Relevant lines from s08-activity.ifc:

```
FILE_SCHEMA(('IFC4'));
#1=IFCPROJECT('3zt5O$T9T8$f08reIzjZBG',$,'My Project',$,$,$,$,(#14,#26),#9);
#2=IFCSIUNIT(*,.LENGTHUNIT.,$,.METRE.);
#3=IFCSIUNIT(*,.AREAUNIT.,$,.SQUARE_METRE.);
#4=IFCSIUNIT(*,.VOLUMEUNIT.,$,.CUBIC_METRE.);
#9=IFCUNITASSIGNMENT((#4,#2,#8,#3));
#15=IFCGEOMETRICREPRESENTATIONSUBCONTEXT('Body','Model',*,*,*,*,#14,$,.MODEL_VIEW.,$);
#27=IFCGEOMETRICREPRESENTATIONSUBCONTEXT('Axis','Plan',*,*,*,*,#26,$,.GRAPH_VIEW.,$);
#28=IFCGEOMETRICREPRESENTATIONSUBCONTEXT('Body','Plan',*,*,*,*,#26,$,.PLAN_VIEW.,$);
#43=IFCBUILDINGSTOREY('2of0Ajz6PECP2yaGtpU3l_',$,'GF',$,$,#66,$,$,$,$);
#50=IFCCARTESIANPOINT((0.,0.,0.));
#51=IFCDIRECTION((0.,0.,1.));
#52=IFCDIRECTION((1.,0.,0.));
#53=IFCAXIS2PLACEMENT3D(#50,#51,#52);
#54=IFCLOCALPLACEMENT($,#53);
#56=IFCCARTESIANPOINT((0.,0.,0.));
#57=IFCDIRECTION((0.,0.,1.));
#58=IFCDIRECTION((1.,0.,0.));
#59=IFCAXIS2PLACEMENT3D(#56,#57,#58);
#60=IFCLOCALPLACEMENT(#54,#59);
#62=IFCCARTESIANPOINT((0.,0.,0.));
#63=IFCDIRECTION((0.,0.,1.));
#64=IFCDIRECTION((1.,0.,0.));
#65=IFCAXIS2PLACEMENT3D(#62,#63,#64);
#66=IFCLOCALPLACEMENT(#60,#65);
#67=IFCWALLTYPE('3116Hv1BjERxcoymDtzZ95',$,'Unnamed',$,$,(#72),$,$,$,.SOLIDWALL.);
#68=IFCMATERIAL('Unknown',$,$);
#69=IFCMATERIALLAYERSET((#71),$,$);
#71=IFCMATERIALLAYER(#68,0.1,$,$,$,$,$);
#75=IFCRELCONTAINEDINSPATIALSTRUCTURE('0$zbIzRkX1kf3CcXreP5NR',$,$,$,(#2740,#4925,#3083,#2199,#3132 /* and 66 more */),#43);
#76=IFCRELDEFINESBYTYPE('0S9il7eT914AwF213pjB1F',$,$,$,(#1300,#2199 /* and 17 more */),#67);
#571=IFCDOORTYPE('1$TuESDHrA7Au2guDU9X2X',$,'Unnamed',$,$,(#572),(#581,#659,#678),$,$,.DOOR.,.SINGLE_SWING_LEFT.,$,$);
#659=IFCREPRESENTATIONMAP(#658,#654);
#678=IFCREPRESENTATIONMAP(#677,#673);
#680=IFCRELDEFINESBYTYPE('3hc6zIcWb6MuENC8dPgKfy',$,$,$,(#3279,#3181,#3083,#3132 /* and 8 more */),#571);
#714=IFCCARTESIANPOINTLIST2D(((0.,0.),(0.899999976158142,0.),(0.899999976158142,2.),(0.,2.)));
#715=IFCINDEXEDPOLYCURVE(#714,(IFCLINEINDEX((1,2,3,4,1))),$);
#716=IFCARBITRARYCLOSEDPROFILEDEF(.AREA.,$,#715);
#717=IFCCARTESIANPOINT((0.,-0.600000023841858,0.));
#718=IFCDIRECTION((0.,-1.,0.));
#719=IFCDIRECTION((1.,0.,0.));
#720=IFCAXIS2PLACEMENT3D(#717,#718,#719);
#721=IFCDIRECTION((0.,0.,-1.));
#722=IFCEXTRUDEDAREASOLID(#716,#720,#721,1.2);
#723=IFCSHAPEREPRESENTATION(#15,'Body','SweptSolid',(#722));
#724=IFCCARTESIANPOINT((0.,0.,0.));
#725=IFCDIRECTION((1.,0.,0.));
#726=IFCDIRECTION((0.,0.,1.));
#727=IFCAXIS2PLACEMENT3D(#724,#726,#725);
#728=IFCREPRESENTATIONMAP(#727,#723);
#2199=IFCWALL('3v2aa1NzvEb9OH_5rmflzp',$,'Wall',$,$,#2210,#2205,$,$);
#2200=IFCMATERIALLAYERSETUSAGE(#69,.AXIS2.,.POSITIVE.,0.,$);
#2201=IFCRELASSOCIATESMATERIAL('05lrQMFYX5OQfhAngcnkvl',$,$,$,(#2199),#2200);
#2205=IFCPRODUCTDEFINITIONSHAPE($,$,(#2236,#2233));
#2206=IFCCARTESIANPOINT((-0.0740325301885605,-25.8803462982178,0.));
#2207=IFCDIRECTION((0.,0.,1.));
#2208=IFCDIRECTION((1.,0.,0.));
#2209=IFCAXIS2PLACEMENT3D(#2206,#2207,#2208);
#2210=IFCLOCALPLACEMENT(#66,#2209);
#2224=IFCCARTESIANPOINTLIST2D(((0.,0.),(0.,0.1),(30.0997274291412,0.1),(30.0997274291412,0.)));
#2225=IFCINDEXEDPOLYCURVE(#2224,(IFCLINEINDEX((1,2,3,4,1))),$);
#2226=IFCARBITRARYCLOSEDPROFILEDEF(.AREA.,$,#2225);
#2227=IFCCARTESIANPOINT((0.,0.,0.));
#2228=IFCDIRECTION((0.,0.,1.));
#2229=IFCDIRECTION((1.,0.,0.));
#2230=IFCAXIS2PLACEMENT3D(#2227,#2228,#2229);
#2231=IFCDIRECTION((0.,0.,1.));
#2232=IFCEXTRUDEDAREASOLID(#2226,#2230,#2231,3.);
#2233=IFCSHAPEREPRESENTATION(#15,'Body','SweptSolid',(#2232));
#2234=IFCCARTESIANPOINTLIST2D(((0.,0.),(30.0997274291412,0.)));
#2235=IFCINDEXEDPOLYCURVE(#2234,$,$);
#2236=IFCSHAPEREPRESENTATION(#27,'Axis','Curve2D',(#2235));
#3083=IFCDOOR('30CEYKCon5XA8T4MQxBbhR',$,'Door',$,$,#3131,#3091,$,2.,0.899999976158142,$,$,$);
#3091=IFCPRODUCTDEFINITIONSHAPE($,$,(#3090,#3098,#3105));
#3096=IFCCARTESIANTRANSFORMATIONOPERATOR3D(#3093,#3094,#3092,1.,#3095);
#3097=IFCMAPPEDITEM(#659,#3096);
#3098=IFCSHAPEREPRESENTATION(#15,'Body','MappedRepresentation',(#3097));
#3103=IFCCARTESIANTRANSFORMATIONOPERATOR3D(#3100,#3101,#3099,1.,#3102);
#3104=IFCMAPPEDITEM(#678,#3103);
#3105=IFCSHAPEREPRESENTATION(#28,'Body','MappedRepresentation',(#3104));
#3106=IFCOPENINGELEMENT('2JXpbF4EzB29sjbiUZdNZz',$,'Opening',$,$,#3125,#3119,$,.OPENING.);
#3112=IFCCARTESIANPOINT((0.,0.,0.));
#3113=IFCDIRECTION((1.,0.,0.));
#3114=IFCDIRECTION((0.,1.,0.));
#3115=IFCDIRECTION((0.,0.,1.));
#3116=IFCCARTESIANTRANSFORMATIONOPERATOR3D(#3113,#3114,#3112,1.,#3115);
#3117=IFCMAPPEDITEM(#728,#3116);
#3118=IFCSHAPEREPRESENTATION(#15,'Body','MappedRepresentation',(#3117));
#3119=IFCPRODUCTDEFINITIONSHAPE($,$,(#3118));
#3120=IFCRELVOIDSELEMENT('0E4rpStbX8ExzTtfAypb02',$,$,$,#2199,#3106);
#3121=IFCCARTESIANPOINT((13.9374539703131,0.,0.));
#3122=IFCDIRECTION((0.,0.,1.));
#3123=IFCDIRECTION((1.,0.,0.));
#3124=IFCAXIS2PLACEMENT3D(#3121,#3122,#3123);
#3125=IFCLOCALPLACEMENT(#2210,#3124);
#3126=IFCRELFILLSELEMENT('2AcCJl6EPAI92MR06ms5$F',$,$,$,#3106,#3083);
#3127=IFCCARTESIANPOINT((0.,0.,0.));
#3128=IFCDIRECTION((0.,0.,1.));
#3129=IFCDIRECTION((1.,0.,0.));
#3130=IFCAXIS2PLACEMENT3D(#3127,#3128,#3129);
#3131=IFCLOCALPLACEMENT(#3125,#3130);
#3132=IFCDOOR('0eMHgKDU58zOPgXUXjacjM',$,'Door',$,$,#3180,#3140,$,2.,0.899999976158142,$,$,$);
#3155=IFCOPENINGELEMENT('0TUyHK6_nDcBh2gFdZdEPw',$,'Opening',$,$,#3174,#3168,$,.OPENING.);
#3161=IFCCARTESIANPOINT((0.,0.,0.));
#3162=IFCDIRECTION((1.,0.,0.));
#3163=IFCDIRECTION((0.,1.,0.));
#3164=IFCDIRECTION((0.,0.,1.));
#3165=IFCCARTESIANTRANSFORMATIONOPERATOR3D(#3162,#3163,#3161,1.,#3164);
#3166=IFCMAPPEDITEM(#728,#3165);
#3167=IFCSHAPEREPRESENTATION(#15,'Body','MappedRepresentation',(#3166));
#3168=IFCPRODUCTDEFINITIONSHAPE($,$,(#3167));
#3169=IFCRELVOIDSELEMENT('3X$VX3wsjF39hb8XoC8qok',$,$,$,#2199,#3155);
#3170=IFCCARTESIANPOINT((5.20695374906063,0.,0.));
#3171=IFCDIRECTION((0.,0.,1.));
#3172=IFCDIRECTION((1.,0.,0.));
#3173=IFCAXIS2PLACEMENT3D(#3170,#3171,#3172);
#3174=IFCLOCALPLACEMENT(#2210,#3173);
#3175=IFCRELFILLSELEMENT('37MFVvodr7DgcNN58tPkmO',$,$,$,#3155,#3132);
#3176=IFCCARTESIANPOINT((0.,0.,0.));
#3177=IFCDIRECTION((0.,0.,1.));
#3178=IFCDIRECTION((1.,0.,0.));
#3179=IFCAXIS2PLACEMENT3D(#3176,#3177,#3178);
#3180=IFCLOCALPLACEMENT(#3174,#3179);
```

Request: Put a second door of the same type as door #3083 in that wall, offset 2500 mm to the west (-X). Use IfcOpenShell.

```python
import ifcopenshell
import ifcopenshell.api.feature
import ifcopenshell.api.geometry
import ifcopenshell.api.root
import ifcopenshell.geom
import ifcopenshell.util.element
import ifcopenshell.util.placement
import ifcopenshell.util.shape

model = ifcopenshell.open("s08-activity.ifc")
settings = ifcopenshell.geom.settings()


def volume(element):
    """Net volume in cubic metres, openings subtracted."""
    shape = ifcopenshell.geom.create_shape(settings, element)
    return ifcopenshell.util.shape.get_volume(shape.geometry)


door = model.by_id(3083)
opening = door.FillsVoids[0].RelatingOpeningElement
wall = opening.VoidsElements[0].RelatingBuildingElement
before = volume(wall)
shift = ifcopenshell.util.placement.get_local_placement(wall.ObjectPlacement)[:3, 0] * -2.5

# copy_class copies the void relationship, type, container and properties, but no geometry.
new_opening = ifcopenshell.api.root.copy_class(model, product=opening)
new_opening.Representation = ifcopenshell.util.element.copy_deep(
    model, opening.Representation, exclude=["IfcGeometricRepresentationContext", "IfcRepresentationMap"]
)
new_door = ifcopenshell.api.root.copy_class(model, product=door)
new_door.Representation = ifcopenshell.util.element.copy_deep(
    model, door.Representation, exclude=["IfcGeometricRepresentationContext", "IfcRepresentationMap"]
)
ifcopenshell.api.feature.add_filling(model, opening=new_opening, element=new_door)

for old, new in ((opening, new_opening), (door, new_door)):
    matrix = ifcopenshell.util.placement.get_local_placement(old.ObjectPlacement)
    matrix[:3, 3] += shift
    ifcopenshell.api.geometry.edit_object_placement(model, product=new, matrix=matrix, is_si=False)

after = volume(wall)

print(f"wall volume {before:.3f} -> {after:.3f} m3")

model.write("s08-activity_rev.ifc")
```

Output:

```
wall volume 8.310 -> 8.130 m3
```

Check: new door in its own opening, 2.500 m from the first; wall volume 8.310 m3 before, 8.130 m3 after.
